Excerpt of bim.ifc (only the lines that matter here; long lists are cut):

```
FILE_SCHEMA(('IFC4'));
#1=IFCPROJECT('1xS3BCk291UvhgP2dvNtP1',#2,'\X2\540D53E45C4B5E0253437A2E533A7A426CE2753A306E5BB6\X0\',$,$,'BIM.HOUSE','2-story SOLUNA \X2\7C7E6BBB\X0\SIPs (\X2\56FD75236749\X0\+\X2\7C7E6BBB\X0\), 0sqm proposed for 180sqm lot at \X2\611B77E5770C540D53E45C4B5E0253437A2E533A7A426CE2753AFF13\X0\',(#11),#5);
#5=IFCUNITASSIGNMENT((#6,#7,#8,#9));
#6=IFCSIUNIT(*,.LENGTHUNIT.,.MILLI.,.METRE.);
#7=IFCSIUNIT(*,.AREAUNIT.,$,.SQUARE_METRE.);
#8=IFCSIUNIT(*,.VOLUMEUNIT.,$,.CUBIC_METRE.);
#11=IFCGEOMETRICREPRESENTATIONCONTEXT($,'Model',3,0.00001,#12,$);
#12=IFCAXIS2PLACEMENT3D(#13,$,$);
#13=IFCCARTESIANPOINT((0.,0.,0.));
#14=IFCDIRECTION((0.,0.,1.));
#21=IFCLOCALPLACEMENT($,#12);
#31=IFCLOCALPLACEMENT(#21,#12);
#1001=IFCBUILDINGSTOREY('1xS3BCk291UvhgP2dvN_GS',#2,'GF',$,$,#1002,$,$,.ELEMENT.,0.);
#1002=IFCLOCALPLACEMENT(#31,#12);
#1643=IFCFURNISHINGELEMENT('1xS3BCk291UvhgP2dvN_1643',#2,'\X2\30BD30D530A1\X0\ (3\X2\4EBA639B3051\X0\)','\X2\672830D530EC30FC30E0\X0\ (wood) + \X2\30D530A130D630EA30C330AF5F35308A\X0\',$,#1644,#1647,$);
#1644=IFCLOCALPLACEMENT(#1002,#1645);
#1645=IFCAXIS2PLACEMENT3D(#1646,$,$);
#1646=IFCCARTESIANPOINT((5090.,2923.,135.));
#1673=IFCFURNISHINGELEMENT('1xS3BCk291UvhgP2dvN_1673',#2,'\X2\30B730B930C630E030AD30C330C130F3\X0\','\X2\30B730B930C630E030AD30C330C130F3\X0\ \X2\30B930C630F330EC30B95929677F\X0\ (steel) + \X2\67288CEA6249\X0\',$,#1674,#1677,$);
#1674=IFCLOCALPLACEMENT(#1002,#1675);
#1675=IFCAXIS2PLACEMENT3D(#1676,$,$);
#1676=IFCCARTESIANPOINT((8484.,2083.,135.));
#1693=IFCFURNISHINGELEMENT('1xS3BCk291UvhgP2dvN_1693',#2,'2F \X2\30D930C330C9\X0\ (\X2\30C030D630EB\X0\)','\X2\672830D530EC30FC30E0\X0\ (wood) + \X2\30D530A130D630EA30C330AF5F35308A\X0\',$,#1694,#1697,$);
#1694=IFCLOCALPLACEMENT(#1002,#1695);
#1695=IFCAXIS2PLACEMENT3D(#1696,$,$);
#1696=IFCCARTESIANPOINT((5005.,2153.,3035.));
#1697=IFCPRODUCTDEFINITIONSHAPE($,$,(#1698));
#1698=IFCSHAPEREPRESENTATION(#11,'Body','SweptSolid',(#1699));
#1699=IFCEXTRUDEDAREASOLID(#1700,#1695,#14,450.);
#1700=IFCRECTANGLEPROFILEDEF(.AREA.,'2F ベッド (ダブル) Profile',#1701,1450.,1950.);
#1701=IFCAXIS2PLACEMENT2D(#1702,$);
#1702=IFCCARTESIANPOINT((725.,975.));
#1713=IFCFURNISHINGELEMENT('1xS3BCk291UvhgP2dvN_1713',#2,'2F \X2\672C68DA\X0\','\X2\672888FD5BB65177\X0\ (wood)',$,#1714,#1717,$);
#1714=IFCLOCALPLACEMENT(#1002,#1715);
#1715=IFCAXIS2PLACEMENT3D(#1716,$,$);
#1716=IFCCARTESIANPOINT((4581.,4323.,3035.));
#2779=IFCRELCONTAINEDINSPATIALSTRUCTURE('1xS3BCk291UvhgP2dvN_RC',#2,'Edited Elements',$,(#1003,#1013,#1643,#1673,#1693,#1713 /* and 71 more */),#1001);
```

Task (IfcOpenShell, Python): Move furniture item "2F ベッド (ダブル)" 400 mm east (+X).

```python
import ifcopenshell
import ifcopenshell.api.geometry
import ifcopenshell.util.placement

model = ifcopenshell.open("bim.ifc")

item = model.by_id(1693)
matrix = ifcopenshell.util.placement.get_local_placement(item.ObjectPlacement)
matrix[0, 3] += 400.0
ifcopenshell.api.geometry.edit_object_placement(model, product=item, matrix=matrix, is_si=False)

print(ifcopenshell.util.placement.get_local_placement(item.ObjectPlacement).round(3) + 0.0)

model.write("bim_edited.ifc")
```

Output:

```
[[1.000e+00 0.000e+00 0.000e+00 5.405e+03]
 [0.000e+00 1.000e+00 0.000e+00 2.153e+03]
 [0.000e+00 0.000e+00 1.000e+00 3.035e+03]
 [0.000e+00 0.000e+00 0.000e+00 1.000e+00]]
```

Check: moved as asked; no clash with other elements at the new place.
